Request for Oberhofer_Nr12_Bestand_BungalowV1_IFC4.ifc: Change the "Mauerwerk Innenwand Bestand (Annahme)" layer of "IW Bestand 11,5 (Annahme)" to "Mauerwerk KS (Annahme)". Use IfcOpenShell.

First a look at what the model holds.

```python
import ifcopenshell
import ifcopenshell.util.element

model = ifcopenshell.open("Oberhofer_Nr12_Bestand_BungalowV1_IFC4.ifc")
print(model.schema)
for layer_set in model.by_type("IfcMaterialLayerSet"):
    if layer_set.LayerSetName == "IW Bestand 11,5 (Annahme)":
        for layer in layer_set.MaterialLayers:
            print(layer.id(), layer.Material and layer.Material.Name, layer.LayerThickness, sep=" | ")
        print(len(ifcopenshell.util.element.get_elements_by_material(model, layer_set)), "elements and types use it")
print(sorted(m.Name for m in model.by_type("IfcMaterial") if m.Name)[:60])
```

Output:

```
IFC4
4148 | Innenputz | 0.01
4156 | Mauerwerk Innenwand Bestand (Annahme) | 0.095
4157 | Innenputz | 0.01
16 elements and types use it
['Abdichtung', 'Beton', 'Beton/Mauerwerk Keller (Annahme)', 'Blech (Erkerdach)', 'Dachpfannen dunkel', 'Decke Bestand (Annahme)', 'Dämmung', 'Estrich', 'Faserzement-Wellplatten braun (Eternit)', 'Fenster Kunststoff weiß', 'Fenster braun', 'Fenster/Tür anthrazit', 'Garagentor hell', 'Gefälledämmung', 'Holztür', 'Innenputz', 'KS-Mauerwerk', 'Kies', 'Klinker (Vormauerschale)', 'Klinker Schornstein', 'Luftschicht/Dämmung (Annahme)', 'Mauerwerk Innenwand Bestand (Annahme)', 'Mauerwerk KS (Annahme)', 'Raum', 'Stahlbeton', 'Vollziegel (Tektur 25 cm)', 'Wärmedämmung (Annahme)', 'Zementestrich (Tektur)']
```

```python
import ifcopenshell
import ifcopenshell.api.material

model = ifcopenshell.open("Oberhofer_Nr12_Bestand_BungalowV1_IFC4.ifc")

layer_set = next(s for s in model.by_type("IfcMaterialLayerSet") if s.LayerSetName == "IW Bestand 11,5 (Annahme)")
layer = next(l for l in layer_set.MaterialLayers if l.Material and l.Material.Name == "Mauerwerk Innenwand Bestand (Annahme)")
material = next(m for m in model.by_type("IfcMaterial") if m.Name == "Mauerwerk KS (Annahme)")

# Point this one layer at the other material; renaming the old one would change it everywhere.
ifcopenshell.api.material.edit_layer(model, layer=layer, attributes={}, material=material)

print([l.Material.Name if l.Material else None for l in layer_set.MaterialLayers])

model.write("Oberhofer_Nr12_Bestand_BungalowV1_IFC4_v2.ifc")
```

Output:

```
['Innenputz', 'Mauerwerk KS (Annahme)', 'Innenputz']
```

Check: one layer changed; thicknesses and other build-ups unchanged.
